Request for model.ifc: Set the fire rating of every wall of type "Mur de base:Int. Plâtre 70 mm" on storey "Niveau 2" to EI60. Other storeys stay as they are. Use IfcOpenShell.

First a look at what the model holds.

```python
import ifcopenshell
import ifcopenshell.util.element

model = ifcopenshell.open("model.ifc")
print(model.schema)
storey = next(s for s in model.by_type("IfcBuildingStorey") if s.Name == "Niveau 2")
walls = [e for e in ifcopenshell.util.element.get_decomposition(storey) if e.is_a("IfcWall")]
seen = {}
for e in walls:
    element_type = ifcopenshell.util.element.get_type(e)
    key = (element_type.Name if element_type != e and element_type else None, ifcopenshell.util.element.get_pset(e, "Pset_WallCommon", "FireRating"))
    seen[key] = seen.get(key, 0) + 1
for (name, value), count in sorted(seen.items(), key=str):
    print(count, "x", name, "|", value)
```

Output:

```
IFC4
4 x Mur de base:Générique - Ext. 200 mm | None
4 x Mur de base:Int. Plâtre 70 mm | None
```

```python
import ifcopenshell
import ifcopenshell.api.pset
import ifcopenshell.util.element

model = ifcopenshell.open("model.ifc")

storey = next(s for s in model.by_type("IfcBuildingStorey") if s.Name == "Niveau 2")
walls = [e for e in ifcopenshell.util.element.get_decomposition(storey) if e.is_a("IfcWall")]

count = 0
for e in walls:
    element_type = ifcopenshell.util.element.get_type(e)
    if element_type in (None, e) or element_type.Name != "Mur de base:Int. Plâtre 70 mm":
        continue
    # add_pset returns the element's existing set when there is one.
    pset = ifcopenshell.api.pset.add_pset(model, product=e, name="Pset_WallCommon")
    ifcopenshell.api.pset.edit_pset(model, pset=pset, properties={"FireRating": "EI60"})
    count += 1

print(count, "walls updated")

model.write("model_edited.ifc")
```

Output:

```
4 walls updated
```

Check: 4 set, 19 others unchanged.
